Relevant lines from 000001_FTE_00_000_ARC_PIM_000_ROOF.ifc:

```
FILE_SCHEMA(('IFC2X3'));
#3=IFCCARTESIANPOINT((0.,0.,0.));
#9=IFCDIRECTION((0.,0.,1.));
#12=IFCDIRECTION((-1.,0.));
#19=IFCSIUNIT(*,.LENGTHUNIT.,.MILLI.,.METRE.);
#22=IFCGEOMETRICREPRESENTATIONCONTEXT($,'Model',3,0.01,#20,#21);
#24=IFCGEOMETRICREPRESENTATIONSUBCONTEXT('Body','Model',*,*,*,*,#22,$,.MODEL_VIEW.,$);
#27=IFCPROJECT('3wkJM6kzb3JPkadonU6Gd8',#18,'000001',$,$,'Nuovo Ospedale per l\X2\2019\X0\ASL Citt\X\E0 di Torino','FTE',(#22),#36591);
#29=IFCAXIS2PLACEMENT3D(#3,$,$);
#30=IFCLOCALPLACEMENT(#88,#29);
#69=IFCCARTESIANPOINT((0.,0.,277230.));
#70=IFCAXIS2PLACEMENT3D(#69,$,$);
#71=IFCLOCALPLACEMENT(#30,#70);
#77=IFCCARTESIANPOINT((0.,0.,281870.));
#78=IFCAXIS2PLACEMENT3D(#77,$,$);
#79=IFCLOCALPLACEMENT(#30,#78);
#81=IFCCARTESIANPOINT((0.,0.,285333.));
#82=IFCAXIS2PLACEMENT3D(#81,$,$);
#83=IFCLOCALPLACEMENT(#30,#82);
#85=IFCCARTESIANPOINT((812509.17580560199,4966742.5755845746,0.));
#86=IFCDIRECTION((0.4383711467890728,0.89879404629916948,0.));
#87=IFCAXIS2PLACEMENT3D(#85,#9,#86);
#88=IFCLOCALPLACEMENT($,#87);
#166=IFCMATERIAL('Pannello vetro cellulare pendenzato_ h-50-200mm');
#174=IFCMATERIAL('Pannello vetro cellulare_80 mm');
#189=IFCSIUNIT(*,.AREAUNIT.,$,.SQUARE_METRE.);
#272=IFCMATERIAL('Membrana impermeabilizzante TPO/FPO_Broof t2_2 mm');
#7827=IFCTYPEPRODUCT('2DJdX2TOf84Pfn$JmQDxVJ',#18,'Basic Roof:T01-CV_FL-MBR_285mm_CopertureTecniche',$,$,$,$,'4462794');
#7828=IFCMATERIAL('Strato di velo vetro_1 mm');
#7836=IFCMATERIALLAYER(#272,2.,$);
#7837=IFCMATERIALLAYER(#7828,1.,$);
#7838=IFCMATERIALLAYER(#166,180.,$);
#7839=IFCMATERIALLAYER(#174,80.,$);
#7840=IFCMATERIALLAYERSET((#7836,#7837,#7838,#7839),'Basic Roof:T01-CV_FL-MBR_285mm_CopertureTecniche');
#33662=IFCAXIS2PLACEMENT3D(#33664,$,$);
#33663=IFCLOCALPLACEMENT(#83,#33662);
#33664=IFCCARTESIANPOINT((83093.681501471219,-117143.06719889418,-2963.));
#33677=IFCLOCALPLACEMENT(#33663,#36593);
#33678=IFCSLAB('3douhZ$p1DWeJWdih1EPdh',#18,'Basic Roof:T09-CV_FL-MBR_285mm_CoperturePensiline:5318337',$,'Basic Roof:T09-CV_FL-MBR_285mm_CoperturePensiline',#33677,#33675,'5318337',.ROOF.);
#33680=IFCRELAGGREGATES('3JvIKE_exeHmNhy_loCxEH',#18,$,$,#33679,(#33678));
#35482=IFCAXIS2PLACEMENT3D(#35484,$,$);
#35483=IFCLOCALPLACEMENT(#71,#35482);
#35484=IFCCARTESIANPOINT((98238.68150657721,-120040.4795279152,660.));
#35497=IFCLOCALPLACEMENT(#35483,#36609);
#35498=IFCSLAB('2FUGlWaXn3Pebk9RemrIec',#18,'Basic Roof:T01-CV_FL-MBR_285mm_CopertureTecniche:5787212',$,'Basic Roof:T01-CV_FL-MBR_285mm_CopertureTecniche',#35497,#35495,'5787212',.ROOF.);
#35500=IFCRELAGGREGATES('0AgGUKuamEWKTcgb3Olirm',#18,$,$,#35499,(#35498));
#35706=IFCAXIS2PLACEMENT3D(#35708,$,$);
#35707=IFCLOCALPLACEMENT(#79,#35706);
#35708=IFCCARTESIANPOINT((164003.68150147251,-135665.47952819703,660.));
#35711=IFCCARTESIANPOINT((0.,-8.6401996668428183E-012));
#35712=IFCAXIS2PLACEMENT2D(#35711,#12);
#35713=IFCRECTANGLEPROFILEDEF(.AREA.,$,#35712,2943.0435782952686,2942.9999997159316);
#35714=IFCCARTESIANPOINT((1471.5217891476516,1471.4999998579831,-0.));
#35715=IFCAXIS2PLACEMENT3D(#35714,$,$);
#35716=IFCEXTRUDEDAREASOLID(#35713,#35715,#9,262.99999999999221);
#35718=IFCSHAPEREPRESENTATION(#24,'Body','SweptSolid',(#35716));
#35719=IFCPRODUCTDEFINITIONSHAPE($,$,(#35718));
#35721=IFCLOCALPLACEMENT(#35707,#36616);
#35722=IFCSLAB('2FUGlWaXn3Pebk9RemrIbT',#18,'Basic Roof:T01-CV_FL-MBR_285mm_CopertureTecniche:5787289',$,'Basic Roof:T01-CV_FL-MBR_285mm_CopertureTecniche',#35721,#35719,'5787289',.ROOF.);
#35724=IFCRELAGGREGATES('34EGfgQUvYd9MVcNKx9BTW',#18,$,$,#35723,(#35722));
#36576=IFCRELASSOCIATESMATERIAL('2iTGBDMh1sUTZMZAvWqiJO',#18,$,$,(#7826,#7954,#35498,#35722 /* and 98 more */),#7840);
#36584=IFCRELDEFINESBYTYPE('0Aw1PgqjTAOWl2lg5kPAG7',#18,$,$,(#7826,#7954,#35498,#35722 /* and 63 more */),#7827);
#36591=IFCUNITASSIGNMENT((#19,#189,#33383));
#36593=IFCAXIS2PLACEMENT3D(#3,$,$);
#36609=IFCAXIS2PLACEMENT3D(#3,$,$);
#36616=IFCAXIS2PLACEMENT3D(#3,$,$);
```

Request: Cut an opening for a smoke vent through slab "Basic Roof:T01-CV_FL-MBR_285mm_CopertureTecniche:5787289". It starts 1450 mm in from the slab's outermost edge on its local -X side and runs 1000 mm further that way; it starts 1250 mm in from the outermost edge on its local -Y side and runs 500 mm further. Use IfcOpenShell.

```python
import numpy as np
import ifcopenshell
import ifcopenshell.api.feature
import ifcopenshell.api.geometry
import ifcopenshell.api.root
import ifcopenshell.geom
import ifcopenshell.util.placement
import ifcopenshell.util.representation
import ifcopenshell.util.shape
import ifcopenshell.util.unit

model = ifcopenshell.open("000001_FTE_00_000_ARC_PIM_000_ROOF.ifc")
unit_scale = ifcopenshell.util.unit.calculate_unit_scale(model)
settings = ifcopenshell.geom.settings()


def volume(element):
    """Net volume in cubic metres, openings subtracted."""
    shape = ifcopenshell.geom.create_shape(settings, element)
    return ifcopenshell.util.shape.get_volume(shape.geometry)


slab = model.by_guid("2FUGlWaXn3Pebk9RemrIbT")
before = volume(slab)

# Extent in the slab's own axes, in metres. The edges named are its -X and -Y sides.
slab_shape = ifcopenshell.geom.create_shape(settings, slab)
vertices = ifcopenshell.util.shape.get_vertices(slab_shape.geometry)
x_min, y_min, bottom = vertices.min(axis=0)
top = vertices[:, 2].max()

opening = ifcopenshell.api.root.create_entity(model, ifc_class="IfcOpeningElement", name="Smoke vent opening")
context = ifcopenshell.util.representation.get_context(model, "Model", "Body", "MODEL_VIEW")
width, depth = 1, 0.5
outline = [(0.0, 0.0), (width, 0.0), (width, depth), (0.0, depth), (0.0, 0.0)]
# Overshoot both faces by 50 mm so the cut is clean.
shape = ifcopenshell.api.geometry.add_slab_representation(
    model, context=context, depth=top - bottom + 0.1, polyline=outline
)
ifcopenshell.api.geometry.assign_representation(model, product=opening, representation=shape)

matrix = ifcopenshell.util.placement.get_local_placement(slab.ObjectPlacement)
matrix[:, 3] = matrix @ np.append(np.array([x_min + 1.45, y_min + 1.25, bottom - 0.05]) / unit_scale, 1.0)
ifcopenshell.api.geometry.edit_object_placement(model, product=opening, matrix=matrix, is_si=False)
ifcopenshell.api.feature.add_feature(model, feature=opening, element=slab)

after = volume(slab)

print(f"slab volume {before:.3f} -> {after:.3f} m3")

model.write("000001_FTE_00_000_ARC_PIM_000_ROOF_edited.ifc")
```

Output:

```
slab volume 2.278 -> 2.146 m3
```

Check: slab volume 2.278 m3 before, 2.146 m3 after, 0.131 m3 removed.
